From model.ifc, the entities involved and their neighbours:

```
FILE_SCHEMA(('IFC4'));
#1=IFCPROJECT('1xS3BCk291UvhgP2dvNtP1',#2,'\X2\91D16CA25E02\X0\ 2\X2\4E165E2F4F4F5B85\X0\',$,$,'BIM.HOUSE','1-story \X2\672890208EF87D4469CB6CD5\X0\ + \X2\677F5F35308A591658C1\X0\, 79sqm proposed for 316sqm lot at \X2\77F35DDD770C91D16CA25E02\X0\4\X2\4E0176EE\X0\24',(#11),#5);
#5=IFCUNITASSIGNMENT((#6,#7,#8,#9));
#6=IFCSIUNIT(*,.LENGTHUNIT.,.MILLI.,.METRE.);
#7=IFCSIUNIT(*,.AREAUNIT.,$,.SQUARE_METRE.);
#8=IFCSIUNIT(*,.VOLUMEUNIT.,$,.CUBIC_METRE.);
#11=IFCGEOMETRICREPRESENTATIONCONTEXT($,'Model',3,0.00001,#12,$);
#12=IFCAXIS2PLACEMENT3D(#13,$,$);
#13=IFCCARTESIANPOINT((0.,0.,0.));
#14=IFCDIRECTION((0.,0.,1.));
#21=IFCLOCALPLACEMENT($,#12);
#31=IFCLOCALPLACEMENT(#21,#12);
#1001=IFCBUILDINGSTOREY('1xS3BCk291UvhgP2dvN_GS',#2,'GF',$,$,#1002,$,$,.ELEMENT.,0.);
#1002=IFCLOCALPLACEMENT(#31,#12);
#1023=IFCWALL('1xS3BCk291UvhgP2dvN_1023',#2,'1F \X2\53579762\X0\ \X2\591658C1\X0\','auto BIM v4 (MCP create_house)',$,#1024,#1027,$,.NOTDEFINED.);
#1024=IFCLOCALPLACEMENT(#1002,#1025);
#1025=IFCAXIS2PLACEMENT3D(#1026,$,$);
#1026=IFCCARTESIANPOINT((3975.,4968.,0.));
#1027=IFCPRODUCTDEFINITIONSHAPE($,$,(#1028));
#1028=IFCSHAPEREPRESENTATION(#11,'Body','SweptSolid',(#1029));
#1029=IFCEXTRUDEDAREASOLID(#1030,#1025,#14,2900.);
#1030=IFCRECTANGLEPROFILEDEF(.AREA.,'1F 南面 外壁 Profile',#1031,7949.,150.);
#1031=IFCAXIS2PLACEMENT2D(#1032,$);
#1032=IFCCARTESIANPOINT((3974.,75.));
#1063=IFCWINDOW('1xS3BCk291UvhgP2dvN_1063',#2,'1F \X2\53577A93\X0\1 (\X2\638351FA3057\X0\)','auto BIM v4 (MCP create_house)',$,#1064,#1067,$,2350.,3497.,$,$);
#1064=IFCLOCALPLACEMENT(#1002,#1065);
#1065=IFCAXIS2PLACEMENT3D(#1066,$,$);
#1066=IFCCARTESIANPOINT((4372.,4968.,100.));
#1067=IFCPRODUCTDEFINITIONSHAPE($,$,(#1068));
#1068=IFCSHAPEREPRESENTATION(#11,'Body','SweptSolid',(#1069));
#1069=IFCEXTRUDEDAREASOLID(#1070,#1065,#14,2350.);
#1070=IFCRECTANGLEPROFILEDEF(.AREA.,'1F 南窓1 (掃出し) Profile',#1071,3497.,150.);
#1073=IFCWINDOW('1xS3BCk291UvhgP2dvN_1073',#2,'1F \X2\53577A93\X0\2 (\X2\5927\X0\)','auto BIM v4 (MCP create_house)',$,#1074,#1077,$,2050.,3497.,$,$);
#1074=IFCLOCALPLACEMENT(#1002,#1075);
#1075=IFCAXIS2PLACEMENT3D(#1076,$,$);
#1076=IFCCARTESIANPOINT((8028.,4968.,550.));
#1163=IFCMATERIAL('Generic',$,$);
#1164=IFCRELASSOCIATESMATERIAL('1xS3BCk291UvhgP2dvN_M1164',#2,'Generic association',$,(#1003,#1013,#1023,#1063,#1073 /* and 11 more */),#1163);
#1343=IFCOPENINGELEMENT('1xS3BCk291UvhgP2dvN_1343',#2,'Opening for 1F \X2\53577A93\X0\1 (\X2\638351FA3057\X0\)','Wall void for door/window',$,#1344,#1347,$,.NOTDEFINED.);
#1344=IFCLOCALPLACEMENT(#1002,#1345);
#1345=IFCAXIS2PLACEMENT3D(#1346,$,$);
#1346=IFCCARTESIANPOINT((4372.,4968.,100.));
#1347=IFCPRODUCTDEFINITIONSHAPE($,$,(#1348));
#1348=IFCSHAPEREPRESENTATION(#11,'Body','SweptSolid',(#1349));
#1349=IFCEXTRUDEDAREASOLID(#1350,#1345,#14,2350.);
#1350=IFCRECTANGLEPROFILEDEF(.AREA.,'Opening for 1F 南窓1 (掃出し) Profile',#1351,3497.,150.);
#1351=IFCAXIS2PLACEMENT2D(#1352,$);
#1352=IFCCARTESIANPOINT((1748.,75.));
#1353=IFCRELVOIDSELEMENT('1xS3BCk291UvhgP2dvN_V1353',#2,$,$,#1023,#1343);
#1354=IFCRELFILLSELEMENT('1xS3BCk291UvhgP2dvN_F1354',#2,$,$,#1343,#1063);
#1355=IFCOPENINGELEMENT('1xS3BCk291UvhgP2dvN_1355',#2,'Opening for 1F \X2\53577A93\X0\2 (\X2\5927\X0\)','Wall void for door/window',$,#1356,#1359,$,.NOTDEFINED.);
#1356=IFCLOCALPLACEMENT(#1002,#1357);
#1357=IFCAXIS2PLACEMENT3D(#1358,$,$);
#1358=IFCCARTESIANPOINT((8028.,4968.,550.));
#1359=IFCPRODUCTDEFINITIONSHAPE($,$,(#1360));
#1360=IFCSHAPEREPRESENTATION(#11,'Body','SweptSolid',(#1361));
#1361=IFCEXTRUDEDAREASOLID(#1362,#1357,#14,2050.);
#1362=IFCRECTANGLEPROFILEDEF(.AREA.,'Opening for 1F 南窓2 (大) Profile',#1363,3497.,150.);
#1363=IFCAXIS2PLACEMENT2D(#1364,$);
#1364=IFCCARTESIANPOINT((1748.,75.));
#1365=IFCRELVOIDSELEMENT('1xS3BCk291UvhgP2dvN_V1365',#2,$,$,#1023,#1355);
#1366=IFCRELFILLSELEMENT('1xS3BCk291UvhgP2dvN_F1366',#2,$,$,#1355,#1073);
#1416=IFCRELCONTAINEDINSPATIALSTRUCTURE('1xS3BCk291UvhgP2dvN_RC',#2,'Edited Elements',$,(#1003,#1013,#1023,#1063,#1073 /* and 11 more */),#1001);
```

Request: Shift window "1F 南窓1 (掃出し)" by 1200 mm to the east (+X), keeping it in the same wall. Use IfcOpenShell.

```python
import ifcopenshell
import ifcopenshell.api.geometry
import ifcopenshell.util.placement
import ifcopenshell.util.unit

model = ifcopenshell.open("model.ifc")
unit_scale = ifcopenshell.util.unit.calculate_unit_scale(model)

window = model.by_guid("1xS3BCk291UvhgP2dvN_1063")
opening = window.FillsVoids[0].RelatingOpeningElement
wall = opening.VoidsElements[0].RelatingBuildingElement

wall_matrix = ifcopenshell.util.placement.get_local_placement(wall.ObjectPlacement)
shift = wall_matrix[:3, 0] * 1.2 / unit_scale
before = ifcopenshell.util.placement.get_local_placement(window.ObjectPlacement)[:3, 3].copy()

# The window is not placed relative to its opening, so move both.
for product in (opening, window):
    matrix = ifcopenshell.util.placement.get_local_placement(product.ObjectPlacement)
    matrix[:3, 3] += shift
    ifcopenshell.api.geometry.edit_object_placement(model, product=product, matrix=matrix, is_si=False)

after = ifcopenshell.util.placement.get_local_placement(window.ObjectPlacement)[:3, 3]
print("window moved by", (after - before).round(3) + 0.0)

model.write("model_v2.ifc")
```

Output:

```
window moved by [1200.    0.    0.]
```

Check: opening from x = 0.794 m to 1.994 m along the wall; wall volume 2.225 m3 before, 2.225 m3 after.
